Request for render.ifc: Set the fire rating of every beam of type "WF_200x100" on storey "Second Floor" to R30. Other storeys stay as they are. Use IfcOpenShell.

First a look at what the model holds.

```python
import ifcopenshell
import ifcopenshell.util.element

model = ifcopenshell.open("render.ifc")
print(model.schema)
storey = next(s for s in model.by_type("IfcBuildingStorey") if s.Name == "Second Floor")
beams = [e for e in ifcopenshell.util.element.get_decomposition(storey) if e.is_a("IfcBeam")]
seen = {}
for e in beams:
    element_type = ifcopenshell.util.element.get_type(e)
    key = (element_type.Name if element_type != e and element_type else None, ifcopenshell.util.element.get_pset(e, "Pset_BeamCommon", "FireRating"))
    seen[key] = seen.get(key, 0) + 1
for (name, value), count in sorted(seen.items(), key=str):
    print(count, "x", name, "|", value)
```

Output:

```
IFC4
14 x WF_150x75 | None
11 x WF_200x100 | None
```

```python
import ifcopenshell
import ifcopenshell.api.pset
import ifcopenshell.util.element

model = ifcopenshell.open("render.ifc")

storey = next(s for s in model.by_type("IfcBuildingStorey") if s.Name == "Second Floor")
beams = [e for e in ifcopenshell.util.element.get_decomposition(storey) if e.is_a("IfcBeam")]

count = 0
for e in beams:
    element_type = ifcopenshell.util.element.get_type(e)
    if element_type in (None, e) or element_type.Name != "WF_200x100":
        continue
    # add_pset returns the element's existing set when there is one.
    pset = ifcopenshell.api.pset.add_pset(model, product=e, name="Pset_BeamCommon")
    ifcopenshell.api.pset.edit_pset(model, pset=pset, properties={"FireRating": "R30"})
    count += 1

print(count, "beams updated")

model.write("render_rev.ifc")
```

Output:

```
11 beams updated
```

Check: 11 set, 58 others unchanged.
